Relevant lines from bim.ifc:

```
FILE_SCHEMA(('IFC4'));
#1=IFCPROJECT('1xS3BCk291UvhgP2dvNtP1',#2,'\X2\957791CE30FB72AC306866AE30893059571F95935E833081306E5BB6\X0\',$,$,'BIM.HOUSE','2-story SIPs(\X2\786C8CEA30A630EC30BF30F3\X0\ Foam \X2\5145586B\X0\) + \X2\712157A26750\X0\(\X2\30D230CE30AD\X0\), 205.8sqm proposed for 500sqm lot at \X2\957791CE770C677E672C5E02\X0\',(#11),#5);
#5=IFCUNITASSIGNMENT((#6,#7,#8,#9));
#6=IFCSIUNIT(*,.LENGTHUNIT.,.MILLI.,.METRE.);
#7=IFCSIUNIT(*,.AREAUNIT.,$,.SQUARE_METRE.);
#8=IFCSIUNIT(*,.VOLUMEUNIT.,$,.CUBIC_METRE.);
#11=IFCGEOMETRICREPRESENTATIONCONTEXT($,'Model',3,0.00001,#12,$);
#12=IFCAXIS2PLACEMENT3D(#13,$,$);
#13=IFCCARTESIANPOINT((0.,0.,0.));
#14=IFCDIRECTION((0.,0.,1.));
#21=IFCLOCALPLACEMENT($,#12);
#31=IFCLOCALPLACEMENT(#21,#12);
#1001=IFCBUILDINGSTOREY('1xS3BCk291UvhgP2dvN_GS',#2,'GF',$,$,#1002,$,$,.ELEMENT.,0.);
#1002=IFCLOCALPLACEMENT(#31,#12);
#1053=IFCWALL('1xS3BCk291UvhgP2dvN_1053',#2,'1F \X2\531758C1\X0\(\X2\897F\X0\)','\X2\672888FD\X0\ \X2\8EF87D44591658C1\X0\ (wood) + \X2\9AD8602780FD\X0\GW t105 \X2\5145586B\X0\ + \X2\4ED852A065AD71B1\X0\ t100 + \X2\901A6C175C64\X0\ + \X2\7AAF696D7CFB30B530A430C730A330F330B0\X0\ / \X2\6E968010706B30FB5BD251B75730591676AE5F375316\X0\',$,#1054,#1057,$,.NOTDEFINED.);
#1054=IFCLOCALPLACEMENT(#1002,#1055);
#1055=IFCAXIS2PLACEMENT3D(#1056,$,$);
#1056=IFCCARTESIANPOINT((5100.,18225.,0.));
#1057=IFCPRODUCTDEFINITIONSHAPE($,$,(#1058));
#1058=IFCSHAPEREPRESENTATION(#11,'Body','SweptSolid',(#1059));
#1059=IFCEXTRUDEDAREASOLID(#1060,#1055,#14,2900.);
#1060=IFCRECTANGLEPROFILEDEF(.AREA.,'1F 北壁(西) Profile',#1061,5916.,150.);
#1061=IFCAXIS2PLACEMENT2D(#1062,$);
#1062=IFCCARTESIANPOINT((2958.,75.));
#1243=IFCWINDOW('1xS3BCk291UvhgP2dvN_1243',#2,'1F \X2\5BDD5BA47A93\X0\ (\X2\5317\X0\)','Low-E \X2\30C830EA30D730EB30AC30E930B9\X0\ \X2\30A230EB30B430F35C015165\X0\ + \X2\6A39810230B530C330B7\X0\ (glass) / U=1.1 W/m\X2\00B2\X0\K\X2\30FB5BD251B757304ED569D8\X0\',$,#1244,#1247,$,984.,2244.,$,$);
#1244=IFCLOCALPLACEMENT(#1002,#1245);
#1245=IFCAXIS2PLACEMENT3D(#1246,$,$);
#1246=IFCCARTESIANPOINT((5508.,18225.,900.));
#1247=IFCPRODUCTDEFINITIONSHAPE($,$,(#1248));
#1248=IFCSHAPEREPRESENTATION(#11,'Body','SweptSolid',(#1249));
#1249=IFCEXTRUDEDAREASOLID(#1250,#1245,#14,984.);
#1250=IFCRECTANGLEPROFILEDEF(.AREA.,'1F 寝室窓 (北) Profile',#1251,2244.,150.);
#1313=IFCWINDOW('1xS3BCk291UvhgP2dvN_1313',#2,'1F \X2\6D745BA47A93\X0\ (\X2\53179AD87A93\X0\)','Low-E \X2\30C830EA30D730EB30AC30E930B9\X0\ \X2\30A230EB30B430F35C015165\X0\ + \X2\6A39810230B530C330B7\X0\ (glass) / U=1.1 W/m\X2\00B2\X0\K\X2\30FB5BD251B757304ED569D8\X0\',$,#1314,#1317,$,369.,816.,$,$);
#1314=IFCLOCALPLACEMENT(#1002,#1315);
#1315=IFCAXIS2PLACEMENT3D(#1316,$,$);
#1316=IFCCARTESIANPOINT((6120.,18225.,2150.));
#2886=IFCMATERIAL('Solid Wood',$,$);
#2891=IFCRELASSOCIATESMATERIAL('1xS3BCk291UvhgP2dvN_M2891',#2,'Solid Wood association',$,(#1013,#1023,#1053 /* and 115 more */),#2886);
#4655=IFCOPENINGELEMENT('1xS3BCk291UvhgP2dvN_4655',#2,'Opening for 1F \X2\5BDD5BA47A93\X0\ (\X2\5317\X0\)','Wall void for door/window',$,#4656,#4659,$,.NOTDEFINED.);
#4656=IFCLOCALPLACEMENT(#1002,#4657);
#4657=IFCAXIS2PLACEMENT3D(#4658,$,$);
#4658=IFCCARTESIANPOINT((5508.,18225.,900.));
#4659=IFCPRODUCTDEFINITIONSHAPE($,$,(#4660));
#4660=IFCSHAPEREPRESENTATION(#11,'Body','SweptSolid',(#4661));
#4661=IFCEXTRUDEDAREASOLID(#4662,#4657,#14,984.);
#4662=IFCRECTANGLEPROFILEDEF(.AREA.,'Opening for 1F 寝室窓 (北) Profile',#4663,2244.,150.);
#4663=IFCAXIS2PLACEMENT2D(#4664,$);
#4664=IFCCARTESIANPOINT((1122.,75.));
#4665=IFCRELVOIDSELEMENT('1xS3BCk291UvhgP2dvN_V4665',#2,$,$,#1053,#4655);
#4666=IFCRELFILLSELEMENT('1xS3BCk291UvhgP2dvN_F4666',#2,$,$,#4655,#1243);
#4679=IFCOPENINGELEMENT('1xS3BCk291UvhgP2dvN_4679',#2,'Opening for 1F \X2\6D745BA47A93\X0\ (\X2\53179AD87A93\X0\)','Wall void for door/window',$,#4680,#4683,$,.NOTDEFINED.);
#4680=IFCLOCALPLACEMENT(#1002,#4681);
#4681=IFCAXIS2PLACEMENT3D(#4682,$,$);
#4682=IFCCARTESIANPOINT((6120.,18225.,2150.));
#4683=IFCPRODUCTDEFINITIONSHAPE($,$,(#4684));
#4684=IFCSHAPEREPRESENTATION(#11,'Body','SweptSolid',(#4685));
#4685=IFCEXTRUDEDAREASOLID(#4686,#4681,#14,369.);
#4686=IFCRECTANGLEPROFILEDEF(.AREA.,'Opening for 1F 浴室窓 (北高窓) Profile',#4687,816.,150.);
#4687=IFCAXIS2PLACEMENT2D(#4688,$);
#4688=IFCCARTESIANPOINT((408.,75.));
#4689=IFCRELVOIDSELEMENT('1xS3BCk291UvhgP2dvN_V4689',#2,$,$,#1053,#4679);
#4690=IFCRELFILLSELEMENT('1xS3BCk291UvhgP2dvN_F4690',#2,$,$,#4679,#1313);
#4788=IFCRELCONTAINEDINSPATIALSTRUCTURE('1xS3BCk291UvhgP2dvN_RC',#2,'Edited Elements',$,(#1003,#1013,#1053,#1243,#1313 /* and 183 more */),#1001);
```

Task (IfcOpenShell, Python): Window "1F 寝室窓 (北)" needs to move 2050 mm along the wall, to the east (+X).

```python
import ifcopenshell
import ifcopenshell.api.geometry
import ifcopenshell.util.placement
import ifcopenshell.util.unit

model = ifcopenshell.open("bim.ifc")
unit_scale = ifcopenshell.util.unit.calculate_unit_scale(model)

window = model.by_guid("1xS3BCk291UvhgP2dvN_1243")
opening = window.FillsVoids[0].RelatingOpeningElement
wall = opening.VoidsElements[0].RelatingBuildingElement

wall_matrix = ifcopenshell.util.placement.get_local_placement(wall.ObjectPlacement)
shift = wall_matrix[:3, 0] * 2.05 / unit_scale
before = ifcopenshell.util.placement.get_local_placement(window.ObjectPlacement)[:3, 3].copy()

# The window is not placed relative to its opening, so move both.
for product in (opening, window):
    matrix = ifcopenshell.util.placement.get_local_placement(product.ObjectPlacement)
    matrix[:3, 3] += shift
    ifcopenshell.api.geometry.edit_object_placement(model, product=product, matrix=matrix, is_si=False)

after = ifcopenshell.util.placement.get_local_placement(window.ObjectPlacement)[:3, 3]
print("window moved by", (after - before).round(3) + 0.0)

model.write("bim-out.ifc")
```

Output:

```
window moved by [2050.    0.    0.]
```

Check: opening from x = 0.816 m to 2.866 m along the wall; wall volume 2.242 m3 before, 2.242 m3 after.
